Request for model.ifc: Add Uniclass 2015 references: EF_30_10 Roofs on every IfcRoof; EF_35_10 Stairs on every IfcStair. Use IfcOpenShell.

First a look at what the model holds.

```python
import ifcopenshell

model = ifcopenshell.open("model.ifc")
print(model.schema)
print("classifications:", [c.Name for c in model.by_type("IfcClassification")])
for ifc_class in ("IfcDoor", "IfcRoof", "IfcStair", "IfcWall", "IfcWindow"):
    print(ifc_class, len(model.by_type(ifc_class)))
```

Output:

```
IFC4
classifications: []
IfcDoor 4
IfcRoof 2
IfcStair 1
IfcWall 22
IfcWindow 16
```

```python
import ifcopenshell
import ifcopenshell.api.classification

model = ifcopenshell.open("model.ifc")

system = ifcopenshell.api.classification.add_classification(model, classification="Uniclass 2015")

codes = {
    "IfcRoof": ("EF_30_10", "Roofs"),
    "IfcStair": ("EF_35_10", "Stairs"),
}
for ifc_class, (code, name) in codes.items():
    products = model.by_type(ifc_class)
    ifcopenshell.api.classification.add_reference(
        model, products=products, classification=system, identification=code, name=name
    )
    print(code, len(products))

model.write("model-out.ifc")
```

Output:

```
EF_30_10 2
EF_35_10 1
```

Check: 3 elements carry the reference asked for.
